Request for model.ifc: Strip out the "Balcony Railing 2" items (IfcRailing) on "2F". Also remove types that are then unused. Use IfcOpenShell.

First a look at what the model holds.

```python
import ifcopenshell
import ifcopenshell.util.element

model = ifcopenshell.open("model.ifc")
print(model.schema)
storey = next(s for s in model.by_type("IfcBuildingStorey") if s.Name == "2F")
railings = [e for e in ifcopenshell.util.element.get_decomposition(storey) if e.is_a("IfcRailing")]
seen = {}
for e in railings:
    element_type = ifcopenshell.util.element.get_type(e)
    name = element_type.Name if element_type not in (None, e) else None
    seen[name] = seen.get(name, 0) + 1
for name, count in sorted(seen.items(), key=str):
    print(count, "x", name)
```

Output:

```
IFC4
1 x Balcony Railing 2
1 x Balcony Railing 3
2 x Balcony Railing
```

```python
import ifcopenshell
import ifcopenshell.api.root
import ifcopenshell.util.element

model = ifcopenshell.open("model.ifc")

storey = next(s for s in model.by_type("IfcBuildingStorey") if s.Name == "2F")
railings = [e for e in ifcopenshell.util.element.get_decomposition(storey) if e.is_a("IfcRailing")]
targets = [e for e in railings if (t := ifcopenshell.util.element.get_type(e)) not in (None, e) and t.Name == "Balcony Railing 2"]
types = {ifcopenshell.util.element.get_type(e) for e in targets} - {None, *targets}

for e in targets:
    ifcopenshell.api.root.remove_product(model, product=e)
print(len(targets), "removed")

unused = [t for t in types if not ifcopenshell.util.element.get_types(t)]
for t in unused:
    ifcopenshell.api.root.remove_product(model, product=t)
print(len(unused), "unused types removed")

model.write("model_rev.ifc")
```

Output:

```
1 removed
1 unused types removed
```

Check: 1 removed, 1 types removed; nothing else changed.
